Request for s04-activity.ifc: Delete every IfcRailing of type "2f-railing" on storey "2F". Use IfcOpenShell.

First a look at what the model holds.

```python
import ifcopenshell
import ifcopenshell.util.element

model = ifcopenshell.open("s04-activity.ifc")
print(model.schema)
storey = next(s for s in model.by_type("IfcBuildingStorey") if s.Name == "2F")
railings = [e for e in ifcopenshell.util.element.get_decomposition(storey) if e.is_a("IfcRailing")]
seen = {}
for e in railings:
    element_type = ifcopenshell.util.element.get_type(e)
    name = element_type.Name if element_type not in (None, e) else None
    seen[name] = seen.get(name, 0) + 1
for name, count in sorted(seen.items(), key=str):
    print(count, "x", name)
```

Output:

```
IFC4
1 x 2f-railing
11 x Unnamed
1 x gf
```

```python
import ifcopenshell
import ifcopenshell.api.root
import ifcopenshell.util.element

model = ifcopenshell.open("s04-activity.ifc")

storey = next(s for s in model.by_type("IfcBuildingStorey") if s.Name == "2F")
railings = [e for e in ifcopenshell.util.element.get_decomposition(storey) if e.is_a("IfcRailing")]
targets = [e for e in railings if (t := ifcopenshell.util.element.get_type(e)) not in (None, e) and t.Name == "2f-railing"]

for e in targets:
    ifcopenshell.api.root.remove_product(model, product=e)
print(len(targets), "removed")

model.write("s04-activity-out.ifc")
```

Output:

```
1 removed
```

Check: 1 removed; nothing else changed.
